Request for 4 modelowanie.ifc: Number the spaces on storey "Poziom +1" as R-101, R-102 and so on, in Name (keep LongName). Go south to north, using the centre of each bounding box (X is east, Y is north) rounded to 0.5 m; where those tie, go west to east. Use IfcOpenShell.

First a look at what the model holds.

```python
import ifcopenshell
import ifcopenshell.util.element
import ifcopenshell.util.placement

model = ifcopenshell.open("4 modelowanie.ifc")
print(model.schema)
storey = next(s for s in model.by_type("IfcBuildingStorey") if s.Name == "Poziom +1")
spaces = [e for e in ifcopenshell.util.element.get_decomposition(storey) if e.is_a("IfcSpace")]
for e in sorted(spaces, key=lambda e: e.id()):
    origin = ifcopenshell.util.placement.get_local_placement(e.ObjectPlacement)[:3, 3]
    print(e.id(), e.Name, e.LongName, origin.round(2) + 0.0, sep=" | ")
```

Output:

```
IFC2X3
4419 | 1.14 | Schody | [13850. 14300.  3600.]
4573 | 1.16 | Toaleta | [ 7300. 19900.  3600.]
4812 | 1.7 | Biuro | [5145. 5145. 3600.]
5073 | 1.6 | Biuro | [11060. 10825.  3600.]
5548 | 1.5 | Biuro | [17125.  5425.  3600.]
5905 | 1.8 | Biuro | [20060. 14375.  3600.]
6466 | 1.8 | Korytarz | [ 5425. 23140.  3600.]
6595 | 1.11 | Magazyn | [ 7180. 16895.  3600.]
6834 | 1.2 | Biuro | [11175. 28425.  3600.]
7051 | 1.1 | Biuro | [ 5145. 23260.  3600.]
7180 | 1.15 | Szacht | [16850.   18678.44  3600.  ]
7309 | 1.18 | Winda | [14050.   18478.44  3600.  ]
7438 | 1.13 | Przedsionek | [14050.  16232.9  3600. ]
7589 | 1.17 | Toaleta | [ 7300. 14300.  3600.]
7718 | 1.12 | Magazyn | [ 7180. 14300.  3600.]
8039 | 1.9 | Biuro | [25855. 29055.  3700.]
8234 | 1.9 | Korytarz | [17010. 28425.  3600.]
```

```python
import ifcopenshell
import ifcopenshell.geom
import ifcopenshell.util.element
import ifcopenshell.util.shape

model = ifcopenshell.open("4 modelowanie.ifc")
settings = ifcopenshell.geom.settings()
settings.set("use-world-coords", True)


def centre(element):
    shape = ifcopenshell.geom.create_shape(settings, element)
    return ifcopenshell.util.shape.get_bbox_centroid(shape.geometry)


storey = next(s for s in model.by_type("IfcBuildingStorey") if s.Name == "Poziom +1")
spaces = [e for e in ifcopenshell.util.element.get_decomposition(storey) if e.is_a("IfcSpace")]

# Insertion points can sit at a corner or the storey origin, so sort by the geometry (in metres).
centres = {e: centre(e) for e in spaces}
spaces.sort(key=lambda e: (round(centres[e][1] / 0.5), centres[e][0]))

for i, e in enumerate(spaces, start=1):
    number = f"R-1{i:02d}"
    e.Name = number
    print(e.id(), number)

model.write("4 modelowanie-out.ifc")
```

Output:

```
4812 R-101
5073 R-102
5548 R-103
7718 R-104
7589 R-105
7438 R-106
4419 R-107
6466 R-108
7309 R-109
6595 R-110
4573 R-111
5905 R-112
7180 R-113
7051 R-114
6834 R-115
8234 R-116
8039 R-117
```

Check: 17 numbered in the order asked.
